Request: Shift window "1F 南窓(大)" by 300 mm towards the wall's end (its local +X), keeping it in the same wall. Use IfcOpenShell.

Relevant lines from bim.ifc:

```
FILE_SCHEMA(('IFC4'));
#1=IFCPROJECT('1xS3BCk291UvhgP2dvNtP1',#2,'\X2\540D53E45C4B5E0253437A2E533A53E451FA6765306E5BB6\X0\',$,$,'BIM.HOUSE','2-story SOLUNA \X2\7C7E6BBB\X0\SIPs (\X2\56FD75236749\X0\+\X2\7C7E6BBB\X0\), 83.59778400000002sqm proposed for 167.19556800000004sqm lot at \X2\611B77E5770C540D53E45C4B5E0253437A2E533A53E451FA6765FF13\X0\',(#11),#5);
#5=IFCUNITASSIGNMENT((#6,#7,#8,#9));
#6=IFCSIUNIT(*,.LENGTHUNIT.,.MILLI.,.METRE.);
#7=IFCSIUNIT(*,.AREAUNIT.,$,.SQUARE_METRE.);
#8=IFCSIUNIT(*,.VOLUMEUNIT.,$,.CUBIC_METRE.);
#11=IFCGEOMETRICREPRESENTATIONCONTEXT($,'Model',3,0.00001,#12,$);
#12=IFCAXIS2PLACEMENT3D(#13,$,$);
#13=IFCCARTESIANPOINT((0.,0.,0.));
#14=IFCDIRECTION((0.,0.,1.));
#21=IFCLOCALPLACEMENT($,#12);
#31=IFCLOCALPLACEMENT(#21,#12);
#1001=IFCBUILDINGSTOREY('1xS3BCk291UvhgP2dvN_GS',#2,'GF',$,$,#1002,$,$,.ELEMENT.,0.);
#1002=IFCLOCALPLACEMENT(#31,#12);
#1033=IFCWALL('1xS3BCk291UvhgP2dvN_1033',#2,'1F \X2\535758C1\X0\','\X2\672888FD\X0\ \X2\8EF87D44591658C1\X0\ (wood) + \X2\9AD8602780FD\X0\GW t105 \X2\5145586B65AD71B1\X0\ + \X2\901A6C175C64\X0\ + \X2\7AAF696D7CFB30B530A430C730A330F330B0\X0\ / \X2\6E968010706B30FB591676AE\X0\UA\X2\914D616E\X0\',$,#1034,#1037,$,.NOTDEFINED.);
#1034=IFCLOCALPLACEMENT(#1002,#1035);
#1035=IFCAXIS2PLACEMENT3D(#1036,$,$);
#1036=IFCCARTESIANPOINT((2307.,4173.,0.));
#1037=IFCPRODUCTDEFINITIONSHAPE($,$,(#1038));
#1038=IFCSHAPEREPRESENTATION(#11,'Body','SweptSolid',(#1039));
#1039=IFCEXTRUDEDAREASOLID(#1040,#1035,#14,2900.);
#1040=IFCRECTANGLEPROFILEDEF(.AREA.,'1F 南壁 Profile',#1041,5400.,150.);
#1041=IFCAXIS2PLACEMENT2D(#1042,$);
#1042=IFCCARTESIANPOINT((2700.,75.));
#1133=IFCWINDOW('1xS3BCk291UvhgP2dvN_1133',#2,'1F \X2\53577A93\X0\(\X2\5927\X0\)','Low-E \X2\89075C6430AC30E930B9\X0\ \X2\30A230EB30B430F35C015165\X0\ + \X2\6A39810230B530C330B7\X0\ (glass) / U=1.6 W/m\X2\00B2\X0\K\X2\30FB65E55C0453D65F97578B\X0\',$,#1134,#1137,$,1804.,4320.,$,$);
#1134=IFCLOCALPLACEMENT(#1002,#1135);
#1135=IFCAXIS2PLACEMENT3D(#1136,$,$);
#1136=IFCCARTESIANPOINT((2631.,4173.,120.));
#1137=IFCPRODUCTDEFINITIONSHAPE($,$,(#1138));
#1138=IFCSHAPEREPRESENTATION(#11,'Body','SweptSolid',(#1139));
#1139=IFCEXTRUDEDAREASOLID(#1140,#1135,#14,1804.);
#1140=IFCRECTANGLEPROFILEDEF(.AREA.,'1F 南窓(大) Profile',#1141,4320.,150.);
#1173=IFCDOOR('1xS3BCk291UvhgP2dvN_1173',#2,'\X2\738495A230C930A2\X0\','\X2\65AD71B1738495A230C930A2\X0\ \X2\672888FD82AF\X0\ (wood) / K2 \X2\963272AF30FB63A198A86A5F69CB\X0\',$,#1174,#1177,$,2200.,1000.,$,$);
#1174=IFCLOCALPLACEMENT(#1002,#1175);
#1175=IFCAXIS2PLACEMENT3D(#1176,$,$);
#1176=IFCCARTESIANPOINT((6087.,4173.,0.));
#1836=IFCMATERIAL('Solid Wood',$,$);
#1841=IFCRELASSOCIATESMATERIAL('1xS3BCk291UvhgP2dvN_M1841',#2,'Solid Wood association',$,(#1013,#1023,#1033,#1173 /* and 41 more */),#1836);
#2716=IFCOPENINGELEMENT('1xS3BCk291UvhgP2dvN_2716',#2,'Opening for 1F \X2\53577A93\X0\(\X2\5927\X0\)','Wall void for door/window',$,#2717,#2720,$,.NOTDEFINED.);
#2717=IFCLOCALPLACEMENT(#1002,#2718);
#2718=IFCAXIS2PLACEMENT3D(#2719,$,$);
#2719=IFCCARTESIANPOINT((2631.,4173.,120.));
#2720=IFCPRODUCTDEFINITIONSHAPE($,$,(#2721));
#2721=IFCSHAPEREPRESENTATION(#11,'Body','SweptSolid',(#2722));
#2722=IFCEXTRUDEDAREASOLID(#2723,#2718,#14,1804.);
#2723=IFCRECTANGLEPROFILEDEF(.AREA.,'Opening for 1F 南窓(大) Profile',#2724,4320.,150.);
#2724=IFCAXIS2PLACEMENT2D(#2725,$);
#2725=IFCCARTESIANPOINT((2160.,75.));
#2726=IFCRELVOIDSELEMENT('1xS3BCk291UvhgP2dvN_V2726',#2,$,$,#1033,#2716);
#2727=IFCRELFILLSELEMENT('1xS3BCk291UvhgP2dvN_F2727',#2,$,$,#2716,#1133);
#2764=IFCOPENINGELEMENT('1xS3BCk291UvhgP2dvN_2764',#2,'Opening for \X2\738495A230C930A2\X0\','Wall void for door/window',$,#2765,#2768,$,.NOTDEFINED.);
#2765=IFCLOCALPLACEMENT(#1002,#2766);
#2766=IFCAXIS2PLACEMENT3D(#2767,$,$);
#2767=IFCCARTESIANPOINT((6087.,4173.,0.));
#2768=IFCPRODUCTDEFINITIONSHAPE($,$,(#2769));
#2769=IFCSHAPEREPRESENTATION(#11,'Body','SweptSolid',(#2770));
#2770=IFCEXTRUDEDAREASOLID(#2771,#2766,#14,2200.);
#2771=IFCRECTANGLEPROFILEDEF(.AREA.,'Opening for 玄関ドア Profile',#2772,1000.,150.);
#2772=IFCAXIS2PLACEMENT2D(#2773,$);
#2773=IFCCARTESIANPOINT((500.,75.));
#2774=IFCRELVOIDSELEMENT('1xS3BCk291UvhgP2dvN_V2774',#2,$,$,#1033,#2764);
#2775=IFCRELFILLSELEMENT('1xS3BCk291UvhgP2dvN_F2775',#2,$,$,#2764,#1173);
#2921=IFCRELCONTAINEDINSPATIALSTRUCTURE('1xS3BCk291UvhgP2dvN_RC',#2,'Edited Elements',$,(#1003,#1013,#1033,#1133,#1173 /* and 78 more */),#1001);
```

```python
import ifcopenshell
import ifcopenshell.api.geometry
import ifcopenshell.util.placement

model = ifcopenshell.open("bim.ifc")

window = model.by_guid("1xS3BCk291UvhgP2dvN_1133")
opening = window.FillsVoids[0].RelatingOpeningElement
wall = opening.VoidsElements[0].RelatingBuildingElement

wall_matrix = ifcopenshell.util.placement.get_local_placement(wall.ObjectPlacement)
shift = wall_matrix[:3, 0] * 300.0
before = ifcopenshell.util.placement.get_local_placement(window.ObjectPlacement)[:3, 3].copy()

# The window is not placed relative to its opening, so move both.
for product in (opening, window):
    matrix = ifcopenshell.util.placement.get_local_placement(product.ObjectPlacement)
    matrix[:3, 3] += shift
    ifcopenshell.api.geometry.edit_object_placement(model, product=product, matrix=matrix, is_si=False)

after = ifcopenshell.util.placement.get_local_placement(window.ObjectPlacement)[:3, 3]
print("window moved by", (after - before).round(3) + 0.0)

model.write("bim_edited.ifc")
```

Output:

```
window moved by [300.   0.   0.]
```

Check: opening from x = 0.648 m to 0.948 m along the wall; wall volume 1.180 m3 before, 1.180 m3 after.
